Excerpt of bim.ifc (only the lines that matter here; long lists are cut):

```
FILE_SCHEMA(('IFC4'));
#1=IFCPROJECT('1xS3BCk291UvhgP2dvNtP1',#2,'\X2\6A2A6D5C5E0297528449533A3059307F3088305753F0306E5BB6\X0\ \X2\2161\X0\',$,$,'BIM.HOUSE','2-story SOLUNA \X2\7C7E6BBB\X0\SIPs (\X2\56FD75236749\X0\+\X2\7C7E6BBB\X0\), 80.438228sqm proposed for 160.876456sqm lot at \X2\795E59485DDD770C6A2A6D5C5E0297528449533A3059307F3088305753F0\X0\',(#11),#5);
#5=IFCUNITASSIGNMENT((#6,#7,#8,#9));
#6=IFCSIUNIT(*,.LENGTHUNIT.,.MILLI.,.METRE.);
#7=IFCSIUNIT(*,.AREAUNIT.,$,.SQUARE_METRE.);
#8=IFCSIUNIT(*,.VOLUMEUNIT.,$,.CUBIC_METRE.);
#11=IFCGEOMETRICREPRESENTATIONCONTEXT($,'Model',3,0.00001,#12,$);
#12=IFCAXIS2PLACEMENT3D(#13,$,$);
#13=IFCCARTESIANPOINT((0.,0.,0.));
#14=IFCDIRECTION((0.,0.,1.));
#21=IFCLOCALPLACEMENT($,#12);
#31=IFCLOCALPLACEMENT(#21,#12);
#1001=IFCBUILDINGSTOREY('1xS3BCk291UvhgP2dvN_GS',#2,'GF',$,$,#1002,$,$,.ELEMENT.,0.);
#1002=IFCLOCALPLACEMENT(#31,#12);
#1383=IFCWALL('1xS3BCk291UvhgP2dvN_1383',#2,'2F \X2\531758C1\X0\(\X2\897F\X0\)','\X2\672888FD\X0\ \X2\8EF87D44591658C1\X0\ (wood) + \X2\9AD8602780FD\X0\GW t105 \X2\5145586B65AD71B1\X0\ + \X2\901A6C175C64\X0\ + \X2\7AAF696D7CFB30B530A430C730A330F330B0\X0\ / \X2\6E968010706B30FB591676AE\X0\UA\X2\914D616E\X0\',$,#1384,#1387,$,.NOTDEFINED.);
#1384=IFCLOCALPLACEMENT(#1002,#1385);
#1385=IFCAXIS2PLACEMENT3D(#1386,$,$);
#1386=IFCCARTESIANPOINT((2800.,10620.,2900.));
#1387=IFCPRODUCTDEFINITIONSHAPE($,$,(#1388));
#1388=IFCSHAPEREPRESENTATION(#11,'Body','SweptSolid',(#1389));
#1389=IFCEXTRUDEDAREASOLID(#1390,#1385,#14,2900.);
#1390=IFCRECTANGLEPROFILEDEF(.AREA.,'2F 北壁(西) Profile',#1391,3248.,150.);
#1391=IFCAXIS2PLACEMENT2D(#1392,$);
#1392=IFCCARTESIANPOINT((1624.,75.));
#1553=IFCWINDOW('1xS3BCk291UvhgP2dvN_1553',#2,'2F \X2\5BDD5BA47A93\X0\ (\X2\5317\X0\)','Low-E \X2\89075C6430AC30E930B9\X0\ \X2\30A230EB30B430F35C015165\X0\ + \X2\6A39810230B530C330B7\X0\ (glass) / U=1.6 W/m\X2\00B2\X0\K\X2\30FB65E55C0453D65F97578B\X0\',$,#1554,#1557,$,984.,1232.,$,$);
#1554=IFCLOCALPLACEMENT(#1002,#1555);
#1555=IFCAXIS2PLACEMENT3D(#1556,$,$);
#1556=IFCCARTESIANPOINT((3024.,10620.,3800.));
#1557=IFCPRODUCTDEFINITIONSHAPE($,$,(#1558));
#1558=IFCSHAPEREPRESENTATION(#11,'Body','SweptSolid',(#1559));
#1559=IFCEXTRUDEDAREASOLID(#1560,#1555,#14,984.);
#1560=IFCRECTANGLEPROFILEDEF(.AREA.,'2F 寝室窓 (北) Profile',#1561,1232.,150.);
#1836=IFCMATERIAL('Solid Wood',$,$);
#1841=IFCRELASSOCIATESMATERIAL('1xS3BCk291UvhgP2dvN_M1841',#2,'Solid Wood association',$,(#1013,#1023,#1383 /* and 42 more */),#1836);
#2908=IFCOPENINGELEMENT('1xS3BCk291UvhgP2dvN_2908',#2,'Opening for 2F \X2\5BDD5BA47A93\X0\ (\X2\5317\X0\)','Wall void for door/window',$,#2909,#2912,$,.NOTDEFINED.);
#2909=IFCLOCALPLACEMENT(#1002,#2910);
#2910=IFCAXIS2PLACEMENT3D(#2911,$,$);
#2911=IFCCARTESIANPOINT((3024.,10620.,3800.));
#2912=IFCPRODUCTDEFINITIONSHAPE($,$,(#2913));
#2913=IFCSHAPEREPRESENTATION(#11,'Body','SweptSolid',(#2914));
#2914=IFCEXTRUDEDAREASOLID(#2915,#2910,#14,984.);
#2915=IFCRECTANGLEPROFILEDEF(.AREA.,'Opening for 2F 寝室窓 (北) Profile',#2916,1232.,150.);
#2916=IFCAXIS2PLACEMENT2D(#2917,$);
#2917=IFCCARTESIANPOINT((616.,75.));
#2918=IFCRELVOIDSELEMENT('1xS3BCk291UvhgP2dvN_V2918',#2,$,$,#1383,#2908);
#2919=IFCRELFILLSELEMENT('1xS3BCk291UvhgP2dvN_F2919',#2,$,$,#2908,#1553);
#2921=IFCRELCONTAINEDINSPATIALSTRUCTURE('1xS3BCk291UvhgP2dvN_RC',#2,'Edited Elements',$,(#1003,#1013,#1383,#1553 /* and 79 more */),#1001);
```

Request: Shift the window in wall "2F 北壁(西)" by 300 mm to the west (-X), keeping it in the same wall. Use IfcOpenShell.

```python
import ifcopenshell
import ifcopenshell.api.geometry
import ifcopenshell.util.placement

model = ifcopenshell.open("bim.ifc")

window = model.by_id(1553)
opening = window.FillsVoids[0].RelatingOpeningElement
wall = opening.VoidsElements[0].RelatingBuildingElement

wall_matrix = ifcopenshell.util.placement.get_local_placement(wall.ObjectPlacement)
shift = wall_matrix[:3, 0] * -300.0
before = ifcopenshell.util.placement.get_local_placement(window.ObjectPlacement)[:3, 3].copy()

# The window is not placed relative to its opening, so move both.
for product in (opening, window):
    matrix = ifcopenshell.util.placement.get_local_placement(product.ObjectPlacement)
    matrix[:3, 3] += shift
    ifcopenshell.api.geometry.edit_object_placement(model, product=product, matrix=matrix, is_si=False)

after = ifcopenshell.util.placement.get_local_placement(window.ObjectPlacement)[:3, 3]
print("window moved by", (after - before).round(3) + 0.0)

model.write("bim_updated.ifc")
```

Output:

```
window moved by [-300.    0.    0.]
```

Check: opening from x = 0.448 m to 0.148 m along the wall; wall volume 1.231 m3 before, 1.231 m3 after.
